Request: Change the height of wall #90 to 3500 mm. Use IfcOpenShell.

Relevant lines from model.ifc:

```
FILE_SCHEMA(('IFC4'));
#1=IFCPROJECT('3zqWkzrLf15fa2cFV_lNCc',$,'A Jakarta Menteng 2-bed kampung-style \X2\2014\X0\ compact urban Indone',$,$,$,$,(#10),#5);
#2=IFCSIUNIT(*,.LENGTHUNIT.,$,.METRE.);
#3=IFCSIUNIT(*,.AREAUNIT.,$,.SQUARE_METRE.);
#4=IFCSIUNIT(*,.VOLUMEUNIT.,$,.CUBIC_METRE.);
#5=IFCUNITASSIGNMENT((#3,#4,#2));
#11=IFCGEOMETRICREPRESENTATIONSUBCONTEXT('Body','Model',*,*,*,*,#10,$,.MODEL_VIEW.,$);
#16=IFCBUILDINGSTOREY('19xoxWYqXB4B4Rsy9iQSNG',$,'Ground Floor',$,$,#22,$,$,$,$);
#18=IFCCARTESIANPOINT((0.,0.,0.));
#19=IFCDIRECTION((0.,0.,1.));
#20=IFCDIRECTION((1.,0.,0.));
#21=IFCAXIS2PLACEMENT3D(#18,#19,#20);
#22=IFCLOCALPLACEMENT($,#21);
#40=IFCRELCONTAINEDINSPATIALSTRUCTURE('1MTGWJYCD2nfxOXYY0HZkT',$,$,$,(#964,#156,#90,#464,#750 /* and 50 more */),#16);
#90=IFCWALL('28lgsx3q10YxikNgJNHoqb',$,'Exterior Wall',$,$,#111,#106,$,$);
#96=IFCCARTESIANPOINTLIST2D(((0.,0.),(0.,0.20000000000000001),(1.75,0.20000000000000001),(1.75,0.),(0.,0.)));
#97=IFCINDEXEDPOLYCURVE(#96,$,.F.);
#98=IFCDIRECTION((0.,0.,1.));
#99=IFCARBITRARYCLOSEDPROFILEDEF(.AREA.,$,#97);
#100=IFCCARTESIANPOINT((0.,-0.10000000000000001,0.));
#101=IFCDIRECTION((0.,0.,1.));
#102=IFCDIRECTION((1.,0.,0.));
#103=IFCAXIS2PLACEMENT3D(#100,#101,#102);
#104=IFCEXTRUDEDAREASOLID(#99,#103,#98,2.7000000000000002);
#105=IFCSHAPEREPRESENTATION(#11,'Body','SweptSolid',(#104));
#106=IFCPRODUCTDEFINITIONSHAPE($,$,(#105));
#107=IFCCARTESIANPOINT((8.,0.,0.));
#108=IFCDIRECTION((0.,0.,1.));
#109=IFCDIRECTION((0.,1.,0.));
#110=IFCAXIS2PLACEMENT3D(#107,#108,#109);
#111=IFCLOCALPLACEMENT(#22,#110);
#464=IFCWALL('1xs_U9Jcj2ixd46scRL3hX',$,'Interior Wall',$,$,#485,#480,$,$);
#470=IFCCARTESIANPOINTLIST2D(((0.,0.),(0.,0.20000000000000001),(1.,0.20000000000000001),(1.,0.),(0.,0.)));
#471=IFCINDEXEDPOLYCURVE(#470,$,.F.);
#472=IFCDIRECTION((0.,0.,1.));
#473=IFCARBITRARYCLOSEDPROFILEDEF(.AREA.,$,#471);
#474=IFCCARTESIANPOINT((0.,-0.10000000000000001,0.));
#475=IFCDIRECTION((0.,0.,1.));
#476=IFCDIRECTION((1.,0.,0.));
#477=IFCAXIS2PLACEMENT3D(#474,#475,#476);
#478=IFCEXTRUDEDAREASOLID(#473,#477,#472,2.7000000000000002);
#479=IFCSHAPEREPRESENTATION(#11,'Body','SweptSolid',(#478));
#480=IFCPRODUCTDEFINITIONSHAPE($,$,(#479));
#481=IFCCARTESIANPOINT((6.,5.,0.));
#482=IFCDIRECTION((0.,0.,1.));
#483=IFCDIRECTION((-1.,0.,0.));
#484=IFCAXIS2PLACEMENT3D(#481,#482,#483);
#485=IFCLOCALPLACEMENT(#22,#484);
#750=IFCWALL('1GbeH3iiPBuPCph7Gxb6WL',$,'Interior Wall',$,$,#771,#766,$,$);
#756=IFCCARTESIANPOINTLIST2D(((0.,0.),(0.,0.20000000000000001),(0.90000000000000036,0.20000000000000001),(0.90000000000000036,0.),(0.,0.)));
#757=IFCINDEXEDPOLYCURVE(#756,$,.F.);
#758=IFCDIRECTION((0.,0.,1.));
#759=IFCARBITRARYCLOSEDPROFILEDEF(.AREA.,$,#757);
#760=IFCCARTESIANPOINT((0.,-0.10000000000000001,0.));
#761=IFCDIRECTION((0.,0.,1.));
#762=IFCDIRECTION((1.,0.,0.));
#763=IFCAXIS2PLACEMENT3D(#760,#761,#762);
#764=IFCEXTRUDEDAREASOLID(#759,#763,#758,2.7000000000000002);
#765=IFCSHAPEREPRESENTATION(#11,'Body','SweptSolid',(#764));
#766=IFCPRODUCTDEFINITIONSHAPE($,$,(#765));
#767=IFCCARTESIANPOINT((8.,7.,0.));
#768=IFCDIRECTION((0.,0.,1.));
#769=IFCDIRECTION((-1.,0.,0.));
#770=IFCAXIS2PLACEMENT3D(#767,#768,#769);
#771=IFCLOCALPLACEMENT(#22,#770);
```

```python
import ifcopenshell
import ifcopenshell.geom
import ifcopenshell.util.representation
import ifcopenshell.util.shape
import ifcopenshell.util.unit

model = ifcopenshell.open("model.ifc")
unit_scale = ifcopenshell.util.unit.calculate_unit_scale(model)
settings = ifcopenshell.geom.settings()


def volume(element):
    """Net volume in cubic metres, openings subtracted."""
    shape = ifcopenshell.geom.create_shape(settings, element)
    return ifcopenshell.util.shape.get_volume(shape.geometry)


wall = model.by_guid("28lgsx3q10YxikNgJNHoqb")
before = volume(wall)

body = ifcopenshell.util.representation.get_representation(wall, "Model", "Body")
solid = body.Items[0]
old_height = solid.Depth
solid.Depth = 3.5 / unit_scale
after = volume(wall)

print(f"height {old_height:g} -> {solid.Depth:g}, volume {before:.3f} -> {after:.3f} m3")

model.write("model_updated.ifc")
```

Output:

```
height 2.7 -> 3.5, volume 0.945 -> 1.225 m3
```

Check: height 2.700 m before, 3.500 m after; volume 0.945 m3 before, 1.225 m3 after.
